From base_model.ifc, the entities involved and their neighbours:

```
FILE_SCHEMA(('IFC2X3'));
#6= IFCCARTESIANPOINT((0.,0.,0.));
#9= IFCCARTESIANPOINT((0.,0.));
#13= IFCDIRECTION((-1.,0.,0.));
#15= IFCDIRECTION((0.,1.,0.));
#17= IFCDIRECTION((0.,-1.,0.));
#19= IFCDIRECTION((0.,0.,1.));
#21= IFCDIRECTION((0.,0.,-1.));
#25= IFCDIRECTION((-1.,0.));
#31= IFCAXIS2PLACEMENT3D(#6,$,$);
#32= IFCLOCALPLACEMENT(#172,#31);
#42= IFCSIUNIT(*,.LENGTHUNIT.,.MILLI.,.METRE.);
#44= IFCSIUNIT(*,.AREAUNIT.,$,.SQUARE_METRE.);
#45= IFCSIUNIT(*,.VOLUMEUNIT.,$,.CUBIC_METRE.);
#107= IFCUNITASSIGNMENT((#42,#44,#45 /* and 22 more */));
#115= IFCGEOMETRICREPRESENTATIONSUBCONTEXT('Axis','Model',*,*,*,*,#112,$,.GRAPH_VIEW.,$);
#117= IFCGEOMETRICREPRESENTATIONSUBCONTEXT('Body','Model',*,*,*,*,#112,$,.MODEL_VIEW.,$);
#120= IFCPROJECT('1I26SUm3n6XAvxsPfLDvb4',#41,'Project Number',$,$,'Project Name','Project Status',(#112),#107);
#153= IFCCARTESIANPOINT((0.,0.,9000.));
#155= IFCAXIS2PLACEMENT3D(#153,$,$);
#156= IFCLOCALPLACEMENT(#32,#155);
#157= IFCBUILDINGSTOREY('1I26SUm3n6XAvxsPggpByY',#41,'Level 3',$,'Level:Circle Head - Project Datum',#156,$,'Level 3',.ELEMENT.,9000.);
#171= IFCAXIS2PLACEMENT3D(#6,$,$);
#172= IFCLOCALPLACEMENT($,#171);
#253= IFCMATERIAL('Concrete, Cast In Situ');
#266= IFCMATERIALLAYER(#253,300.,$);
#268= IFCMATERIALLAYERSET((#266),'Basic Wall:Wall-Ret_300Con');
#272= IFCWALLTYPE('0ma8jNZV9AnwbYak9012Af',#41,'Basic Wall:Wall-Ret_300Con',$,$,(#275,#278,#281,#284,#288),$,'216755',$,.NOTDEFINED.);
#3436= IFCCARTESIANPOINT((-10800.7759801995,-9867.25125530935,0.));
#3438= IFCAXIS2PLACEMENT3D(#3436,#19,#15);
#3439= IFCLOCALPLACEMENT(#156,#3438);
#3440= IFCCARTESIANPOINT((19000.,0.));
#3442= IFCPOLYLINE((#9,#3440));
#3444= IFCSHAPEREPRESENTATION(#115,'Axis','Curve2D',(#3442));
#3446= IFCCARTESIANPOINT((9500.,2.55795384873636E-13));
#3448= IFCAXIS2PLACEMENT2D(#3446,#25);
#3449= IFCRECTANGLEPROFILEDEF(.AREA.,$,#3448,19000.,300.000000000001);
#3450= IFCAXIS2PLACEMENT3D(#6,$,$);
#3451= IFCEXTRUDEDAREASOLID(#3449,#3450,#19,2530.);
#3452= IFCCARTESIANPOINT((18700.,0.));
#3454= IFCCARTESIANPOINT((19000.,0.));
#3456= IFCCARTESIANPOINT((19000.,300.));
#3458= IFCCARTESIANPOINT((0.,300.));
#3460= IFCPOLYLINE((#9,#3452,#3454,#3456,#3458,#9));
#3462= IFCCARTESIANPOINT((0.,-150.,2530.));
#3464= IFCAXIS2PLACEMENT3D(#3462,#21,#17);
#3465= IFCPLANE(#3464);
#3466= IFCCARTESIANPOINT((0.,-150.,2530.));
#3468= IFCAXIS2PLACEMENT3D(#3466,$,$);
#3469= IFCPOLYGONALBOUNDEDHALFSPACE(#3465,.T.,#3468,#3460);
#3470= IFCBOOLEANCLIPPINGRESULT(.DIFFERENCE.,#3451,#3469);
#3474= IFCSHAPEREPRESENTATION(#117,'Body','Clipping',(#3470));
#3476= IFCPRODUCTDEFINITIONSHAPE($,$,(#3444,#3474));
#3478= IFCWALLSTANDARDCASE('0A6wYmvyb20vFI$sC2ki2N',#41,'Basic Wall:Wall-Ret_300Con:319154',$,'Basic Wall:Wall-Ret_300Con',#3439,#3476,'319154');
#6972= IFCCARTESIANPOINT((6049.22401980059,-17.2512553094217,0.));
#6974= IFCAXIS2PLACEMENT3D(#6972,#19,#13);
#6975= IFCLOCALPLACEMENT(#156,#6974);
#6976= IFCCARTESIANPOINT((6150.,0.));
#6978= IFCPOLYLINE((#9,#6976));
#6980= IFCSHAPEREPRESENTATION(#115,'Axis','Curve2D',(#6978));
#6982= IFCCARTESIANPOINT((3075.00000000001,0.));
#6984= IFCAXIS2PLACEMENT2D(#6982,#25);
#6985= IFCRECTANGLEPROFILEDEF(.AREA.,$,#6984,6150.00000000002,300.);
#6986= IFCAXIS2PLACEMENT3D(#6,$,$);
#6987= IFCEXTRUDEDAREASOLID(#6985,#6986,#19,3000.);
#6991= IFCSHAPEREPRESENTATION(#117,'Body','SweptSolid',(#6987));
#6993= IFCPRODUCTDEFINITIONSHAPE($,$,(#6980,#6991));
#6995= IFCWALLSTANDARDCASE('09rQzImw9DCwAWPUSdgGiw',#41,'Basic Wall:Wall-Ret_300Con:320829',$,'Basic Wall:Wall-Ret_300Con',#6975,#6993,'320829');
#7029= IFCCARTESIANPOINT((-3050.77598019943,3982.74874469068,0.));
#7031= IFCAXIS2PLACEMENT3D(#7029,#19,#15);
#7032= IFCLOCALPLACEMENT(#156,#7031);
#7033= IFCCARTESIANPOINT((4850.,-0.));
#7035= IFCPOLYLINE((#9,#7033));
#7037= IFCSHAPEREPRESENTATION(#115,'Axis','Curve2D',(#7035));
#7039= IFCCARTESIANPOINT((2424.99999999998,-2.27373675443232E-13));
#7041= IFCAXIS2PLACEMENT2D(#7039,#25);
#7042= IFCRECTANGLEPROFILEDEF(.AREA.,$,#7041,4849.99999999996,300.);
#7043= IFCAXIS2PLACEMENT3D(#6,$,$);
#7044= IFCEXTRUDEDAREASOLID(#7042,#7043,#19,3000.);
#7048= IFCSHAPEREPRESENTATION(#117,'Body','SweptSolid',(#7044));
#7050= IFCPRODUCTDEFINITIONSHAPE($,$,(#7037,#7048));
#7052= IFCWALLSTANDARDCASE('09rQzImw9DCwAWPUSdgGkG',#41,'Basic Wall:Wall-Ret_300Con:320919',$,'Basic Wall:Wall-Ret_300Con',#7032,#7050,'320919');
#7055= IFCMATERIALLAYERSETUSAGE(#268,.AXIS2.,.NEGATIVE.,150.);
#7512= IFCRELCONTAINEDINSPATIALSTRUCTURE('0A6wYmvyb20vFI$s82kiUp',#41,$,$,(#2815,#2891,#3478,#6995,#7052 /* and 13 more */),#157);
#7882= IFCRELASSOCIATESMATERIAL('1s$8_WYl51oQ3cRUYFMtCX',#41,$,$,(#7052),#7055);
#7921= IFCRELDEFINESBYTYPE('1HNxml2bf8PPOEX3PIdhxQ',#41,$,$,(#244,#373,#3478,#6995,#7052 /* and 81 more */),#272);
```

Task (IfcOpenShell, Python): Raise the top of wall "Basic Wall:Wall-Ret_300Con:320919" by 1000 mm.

```python
import ifcopenshell
import ifcopenshell.geom
import ifcopenshell.util.representation
import ifcopenshell.util.shape
import ifcopenshell.util.unit

model = ifcopenshell.open("base_model.ifc")
unit_scale = ifcopenshell.util.unit.calculate_unit_scale(model)
settings = ifcopenshell.geom.settings()


def volume(element):
    """Net volume in cubic metres, openings subtracted."""
    shape = ifcopenshell.geom.create_shape(settings, element)
    return ifcopenshell.util.shape.get_volume(shape.geometry)


wall = model.by_guid("09rQzImw9DCwAWPUSdgGkG")
before = volume(wall)

body = ifcopenshell.util.representation.get_representation(wall, "Model", "Body")
solid = body.Items[0]
old_height = solid.Depth
solid.Depth += 1 / unit_scale
after = volume(wall)

print(f"height {old_height:g} -> {solid.Depth:g}, volume {before:.3f} -> {after:.3f} m3")

model.write("base_model_edited.ifc")
```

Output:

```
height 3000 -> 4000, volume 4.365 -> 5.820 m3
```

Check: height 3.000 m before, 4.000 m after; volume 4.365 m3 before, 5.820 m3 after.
